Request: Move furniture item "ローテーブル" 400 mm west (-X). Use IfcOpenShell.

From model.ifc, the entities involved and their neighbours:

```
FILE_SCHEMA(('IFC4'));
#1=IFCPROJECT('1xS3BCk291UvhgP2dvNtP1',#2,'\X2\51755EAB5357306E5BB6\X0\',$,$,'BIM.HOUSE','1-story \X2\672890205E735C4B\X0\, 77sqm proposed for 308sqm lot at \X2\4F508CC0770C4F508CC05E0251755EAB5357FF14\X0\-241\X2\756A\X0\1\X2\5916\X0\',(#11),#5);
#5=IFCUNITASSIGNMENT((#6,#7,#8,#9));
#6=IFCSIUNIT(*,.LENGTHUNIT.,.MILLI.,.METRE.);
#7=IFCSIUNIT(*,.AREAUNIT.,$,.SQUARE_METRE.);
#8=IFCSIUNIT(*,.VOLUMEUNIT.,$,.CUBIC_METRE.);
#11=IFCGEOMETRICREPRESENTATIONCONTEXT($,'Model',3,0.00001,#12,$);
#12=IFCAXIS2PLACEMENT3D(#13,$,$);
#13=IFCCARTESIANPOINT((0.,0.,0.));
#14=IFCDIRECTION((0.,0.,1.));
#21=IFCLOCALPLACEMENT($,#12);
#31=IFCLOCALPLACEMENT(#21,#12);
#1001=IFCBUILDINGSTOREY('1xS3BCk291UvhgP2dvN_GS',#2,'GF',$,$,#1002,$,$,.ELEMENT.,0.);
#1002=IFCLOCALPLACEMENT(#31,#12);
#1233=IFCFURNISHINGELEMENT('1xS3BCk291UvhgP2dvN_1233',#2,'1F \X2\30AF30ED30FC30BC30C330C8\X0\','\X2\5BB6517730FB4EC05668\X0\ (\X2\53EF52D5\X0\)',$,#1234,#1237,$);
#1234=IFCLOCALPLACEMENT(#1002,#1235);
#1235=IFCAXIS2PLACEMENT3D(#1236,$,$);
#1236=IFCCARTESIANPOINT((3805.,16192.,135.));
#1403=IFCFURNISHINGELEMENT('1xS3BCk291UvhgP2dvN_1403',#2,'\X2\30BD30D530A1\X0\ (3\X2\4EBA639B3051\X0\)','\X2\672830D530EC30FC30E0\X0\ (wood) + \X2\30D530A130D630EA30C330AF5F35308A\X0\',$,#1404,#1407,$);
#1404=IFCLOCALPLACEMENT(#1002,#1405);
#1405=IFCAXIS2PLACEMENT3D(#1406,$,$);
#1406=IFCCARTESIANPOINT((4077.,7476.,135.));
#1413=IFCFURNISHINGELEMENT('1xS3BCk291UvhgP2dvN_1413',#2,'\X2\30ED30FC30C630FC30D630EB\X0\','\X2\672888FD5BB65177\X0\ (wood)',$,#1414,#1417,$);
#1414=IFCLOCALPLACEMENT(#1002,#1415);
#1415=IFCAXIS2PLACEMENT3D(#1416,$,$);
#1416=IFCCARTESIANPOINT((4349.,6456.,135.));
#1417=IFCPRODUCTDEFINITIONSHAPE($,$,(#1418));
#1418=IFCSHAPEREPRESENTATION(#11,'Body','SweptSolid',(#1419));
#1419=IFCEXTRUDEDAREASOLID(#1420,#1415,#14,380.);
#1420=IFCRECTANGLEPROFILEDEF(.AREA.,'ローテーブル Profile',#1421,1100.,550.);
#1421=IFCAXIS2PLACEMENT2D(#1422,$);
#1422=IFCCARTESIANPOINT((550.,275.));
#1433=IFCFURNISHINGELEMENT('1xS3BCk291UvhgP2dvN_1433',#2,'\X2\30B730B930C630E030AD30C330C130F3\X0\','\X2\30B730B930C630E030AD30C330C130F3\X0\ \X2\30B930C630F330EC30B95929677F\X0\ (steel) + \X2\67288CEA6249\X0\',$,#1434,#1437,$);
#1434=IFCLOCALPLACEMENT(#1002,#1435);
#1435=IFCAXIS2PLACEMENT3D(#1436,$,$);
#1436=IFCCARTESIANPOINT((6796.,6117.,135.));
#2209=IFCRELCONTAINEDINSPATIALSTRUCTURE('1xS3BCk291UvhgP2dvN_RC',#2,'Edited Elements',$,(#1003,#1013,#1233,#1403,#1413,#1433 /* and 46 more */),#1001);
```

```python
import ifcopenshell
import ifcopenshell.api.geometry
import ifcopenshell.util.placement

model = ifcopenshell.open("model.ifc")

item = model.by_id(1413)
matrix = ifcopenshell.util.placement.get_local_placement(item.ObjectPlacement)
matrix[0, 3] -= 400.0
ifcopenshell.api.geometry.edit_object_placement(model, product=item, matrix=matrix, is_si=False)

print(ifcopenshell.util.placement.get_local_placement(item.ObjectPlacement).round(3) + 0.0)

model.write("model_updated.ifc")
```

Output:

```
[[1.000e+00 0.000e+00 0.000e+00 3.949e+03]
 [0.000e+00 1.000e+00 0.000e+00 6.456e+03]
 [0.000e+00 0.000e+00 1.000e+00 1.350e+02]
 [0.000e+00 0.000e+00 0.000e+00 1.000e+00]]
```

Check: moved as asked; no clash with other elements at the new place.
